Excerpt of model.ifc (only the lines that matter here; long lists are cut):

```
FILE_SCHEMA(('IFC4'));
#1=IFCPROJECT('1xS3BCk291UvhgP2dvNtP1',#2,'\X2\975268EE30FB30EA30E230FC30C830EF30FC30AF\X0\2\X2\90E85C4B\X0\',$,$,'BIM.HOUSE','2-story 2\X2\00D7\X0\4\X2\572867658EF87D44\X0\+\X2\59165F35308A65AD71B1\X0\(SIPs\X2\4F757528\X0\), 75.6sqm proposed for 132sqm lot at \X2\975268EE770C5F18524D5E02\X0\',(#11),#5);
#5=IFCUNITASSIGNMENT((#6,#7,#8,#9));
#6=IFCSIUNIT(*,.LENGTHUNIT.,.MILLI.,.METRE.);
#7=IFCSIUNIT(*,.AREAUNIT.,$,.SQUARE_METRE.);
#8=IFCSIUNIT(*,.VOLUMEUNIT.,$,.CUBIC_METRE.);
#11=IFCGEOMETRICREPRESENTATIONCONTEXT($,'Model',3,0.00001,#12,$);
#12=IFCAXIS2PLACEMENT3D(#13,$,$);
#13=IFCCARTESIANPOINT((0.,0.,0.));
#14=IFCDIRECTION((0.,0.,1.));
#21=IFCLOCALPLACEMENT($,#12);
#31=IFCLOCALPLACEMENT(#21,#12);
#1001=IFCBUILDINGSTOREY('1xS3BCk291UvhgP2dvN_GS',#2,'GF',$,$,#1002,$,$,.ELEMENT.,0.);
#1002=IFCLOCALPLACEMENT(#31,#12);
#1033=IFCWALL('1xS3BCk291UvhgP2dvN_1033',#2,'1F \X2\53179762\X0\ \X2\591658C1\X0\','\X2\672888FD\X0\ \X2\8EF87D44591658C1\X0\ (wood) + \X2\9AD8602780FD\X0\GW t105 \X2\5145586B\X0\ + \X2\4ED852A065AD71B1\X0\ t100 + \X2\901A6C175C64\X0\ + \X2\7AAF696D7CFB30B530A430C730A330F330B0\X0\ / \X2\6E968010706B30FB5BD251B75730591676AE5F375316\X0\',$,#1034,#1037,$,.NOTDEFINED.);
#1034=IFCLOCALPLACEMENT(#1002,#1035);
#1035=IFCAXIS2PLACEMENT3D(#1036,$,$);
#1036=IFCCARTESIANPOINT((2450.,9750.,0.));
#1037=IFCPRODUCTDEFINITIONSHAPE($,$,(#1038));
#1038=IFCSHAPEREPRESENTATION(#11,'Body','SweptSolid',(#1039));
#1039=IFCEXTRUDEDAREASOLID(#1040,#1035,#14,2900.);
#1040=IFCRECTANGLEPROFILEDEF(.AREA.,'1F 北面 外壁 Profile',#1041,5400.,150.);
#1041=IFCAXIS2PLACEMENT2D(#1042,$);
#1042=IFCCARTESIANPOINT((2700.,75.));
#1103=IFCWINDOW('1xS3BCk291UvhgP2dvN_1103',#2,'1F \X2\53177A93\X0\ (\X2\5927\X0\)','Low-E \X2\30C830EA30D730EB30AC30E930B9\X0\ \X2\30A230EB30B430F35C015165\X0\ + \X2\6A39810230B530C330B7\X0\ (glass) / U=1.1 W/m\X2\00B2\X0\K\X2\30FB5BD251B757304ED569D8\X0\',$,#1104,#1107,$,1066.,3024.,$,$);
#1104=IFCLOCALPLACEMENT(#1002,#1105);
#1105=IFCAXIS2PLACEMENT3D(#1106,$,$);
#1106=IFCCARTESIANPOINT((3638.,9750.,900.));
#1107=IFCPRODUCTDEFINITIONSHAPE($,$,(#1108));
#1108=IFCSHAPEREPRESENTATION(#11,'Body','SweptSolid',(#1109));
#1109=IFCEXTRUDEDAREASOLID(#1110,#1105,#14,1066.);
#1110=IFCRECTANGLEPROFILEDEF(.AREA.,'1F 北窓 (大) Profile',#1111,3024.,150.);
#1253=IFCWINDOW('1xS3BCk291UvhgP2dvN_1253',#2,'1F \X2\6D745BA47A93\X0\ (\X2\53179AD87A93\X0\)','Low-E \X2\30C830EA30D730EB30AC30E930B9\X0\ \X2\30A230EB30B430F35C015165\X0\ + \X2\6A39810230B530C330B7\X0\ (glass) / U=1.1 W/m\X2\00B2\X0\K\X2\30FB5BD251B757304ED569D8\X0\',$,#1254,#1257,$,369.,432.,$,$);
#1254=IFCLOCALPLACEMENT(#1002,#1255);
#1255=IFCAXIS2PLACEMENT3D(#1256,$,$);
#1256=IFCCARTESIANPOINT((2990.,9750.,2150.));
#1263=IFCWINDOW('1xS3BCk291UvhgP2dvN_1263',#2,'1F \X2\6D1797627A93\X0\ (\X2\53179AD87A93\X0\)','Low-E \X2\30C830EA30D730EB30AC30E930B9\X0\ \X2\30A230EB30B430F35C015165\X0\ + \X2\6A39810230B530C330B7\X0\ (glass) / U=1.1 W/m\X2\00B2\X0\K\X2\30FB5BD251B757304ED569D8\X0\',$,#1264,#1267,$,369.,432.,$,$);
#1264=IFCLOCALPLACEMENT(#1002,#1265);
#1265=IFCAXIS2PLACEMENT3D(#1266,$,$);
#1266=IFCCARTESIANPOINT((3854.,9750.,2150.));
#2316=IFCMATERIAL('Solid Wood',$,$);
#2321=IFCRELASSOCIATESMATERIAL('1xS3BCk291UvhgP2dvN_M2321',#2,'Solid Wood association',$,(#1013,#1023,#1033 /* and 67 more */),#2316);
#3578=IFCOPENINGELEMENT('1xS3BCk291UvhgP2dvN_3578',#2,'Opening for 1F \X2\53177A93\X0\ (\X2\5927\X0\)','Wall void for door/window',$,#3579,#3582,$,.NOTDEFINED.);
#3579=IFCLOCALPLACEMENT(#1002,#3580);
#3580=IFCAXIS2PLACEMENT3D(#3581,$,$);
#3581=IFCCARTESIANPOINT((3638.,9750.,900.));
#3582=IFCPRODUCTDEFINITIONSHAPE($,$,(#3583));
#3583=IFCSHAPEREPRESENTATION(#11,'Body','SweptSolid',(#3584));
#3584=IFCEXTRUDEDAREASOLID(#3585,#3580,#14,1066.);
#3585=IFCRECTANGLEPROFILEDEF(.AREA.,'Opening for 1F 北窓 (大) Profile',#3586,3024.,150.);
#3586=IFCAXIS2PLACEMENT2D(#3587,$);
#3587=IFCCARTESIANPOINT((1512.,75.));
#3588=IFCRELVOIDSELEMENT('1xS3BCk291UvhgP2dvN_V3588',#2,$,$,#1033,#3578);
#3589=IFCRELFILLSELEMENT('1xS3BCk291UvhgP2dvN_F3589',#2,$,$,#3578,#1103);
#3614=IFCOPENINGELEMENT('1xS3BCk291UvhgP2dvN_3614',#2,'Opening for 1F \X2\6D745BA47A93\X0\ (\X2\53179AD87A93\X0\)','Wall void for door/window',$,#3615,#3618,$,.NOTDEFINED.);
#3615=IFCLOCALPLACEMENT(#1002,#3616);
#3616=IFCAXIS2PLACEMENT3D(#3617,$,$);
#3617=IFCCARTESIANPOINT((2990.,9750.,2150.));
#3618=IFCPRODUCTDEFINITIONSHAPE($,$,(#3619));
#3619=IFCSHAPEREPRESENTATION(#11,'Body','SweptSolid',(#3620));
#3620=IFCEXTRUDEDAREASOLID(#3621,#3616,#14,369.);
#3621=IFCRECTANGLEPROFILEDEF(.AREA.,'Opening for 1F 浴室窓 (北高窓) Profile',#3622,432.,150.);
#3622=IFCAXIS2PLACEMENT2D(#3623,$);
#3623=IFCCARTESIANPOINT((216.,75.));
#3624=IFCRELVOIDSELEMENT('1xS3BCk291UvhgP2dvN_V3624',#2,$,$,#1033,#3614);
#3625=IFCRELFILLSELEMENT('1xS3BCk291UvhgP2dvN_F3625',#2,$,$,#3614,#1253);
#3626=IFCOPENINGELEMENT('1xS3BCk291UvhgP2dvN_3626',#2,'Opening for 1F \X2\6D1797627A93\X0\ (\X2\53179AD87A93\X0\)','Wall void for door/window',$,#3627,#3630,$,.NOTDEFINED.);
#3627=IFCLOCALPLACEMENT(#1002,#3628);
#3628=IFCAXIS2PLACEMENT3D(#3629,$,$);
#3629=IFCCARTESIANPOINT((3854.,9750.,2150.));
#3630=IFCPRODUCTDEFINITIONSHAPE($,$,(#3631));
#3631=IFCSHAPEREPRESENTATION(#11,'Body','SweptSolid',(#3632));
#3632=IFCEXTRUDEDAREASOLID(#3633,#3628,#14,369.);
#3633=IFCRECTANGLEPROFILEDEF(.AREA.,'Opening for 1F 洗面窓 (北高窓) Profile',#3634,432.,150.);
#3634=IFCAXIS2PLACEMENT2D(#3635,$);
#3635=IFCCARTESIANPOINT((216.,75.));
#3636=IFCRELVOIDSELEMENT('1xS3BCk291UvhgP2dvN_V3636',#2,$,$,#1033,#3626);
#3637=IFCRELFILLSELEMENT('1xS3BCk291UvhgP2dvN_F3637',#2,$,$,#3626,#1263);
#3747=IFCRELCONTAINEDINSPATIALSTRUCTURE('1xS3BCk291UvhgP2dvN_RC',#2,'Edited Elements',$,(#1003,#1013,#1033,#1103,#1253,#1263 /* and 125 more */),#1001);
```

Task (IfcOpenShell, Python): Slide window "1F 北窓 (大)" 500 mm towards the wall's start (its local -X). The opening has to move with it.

```python
import ifcopenshell
import ifcopenshell.api.geometry
import ifcopenshell.util.placement
import ifcopenshell.util.unit

model = ifcopenshell.open("model.ifc")
unit_scale = ifcopenshell.util.unit.calculate_unit_scale(model)

window = model.by_id(1103)
opening = window.FillsVoids[0].RelatingOpeningElement
wall = opening.VoidsElements[0].RelatingBuildingElement

wall_matrix = ifcopenshell.util.placement.get_local_placement(wall.ObjectPlacement)
shift = wall_matrix[:3, 0] * -0.5 / unit_scale
before = ifcopenshell.util.placement.get_local_placement(window.ObjectPlacement)[:3, 3].copy()

# The window is not placed relative to its opening, so move both.
for product in (opening, window):
    matrix = ifcopenshell.util.placement.get_local_placement(product.ObjectPlacement)
    matrix[:3, 3] += shift
    ifcopenshell.api.geometry.edit_object_placement(model, product=product, matrix=matrix, is_si=False)

after = ifcopenshell.util.placement.get_local_placement(window.ObjectPlacement)[:3, 3]
print("window moved by", (after - before).round(3) + 0.0)

model.write("model_updated.ifc")
```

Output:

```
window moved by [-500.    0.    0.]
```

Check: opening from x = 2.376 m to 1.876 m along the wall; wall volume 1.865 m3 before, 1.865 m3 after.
